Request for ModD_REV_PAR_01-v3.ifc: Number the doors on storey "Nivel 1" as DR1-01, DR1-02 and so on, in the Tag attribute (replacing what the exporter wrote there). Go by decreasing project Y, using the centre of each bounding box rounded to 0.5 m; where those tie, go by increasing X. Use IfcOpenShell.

First a look at what the model holds.

```python
import ifcopenshell
import ifcopenshell.util.element
import ifcopenshell.util.placement

model = ifcopenshell.open("ModD_REV_PAR_01-v3.ifc")
print(model.schema)
storey = next(s for s in model.by_type("IfcBuildingStorey") if s.Name == "Nivel 1")
doors = [e for e in ifcopenshell.util.element.get_decomposition(storey) if e.is_a("IfcDoor")]
for e in sorted(doors, key=lambda e: e.id()):
    origin = ifcopenshell.util.placement.get_local_placement(e.ObjectPlacement)[:3, 3]
    print(e.id(), e.Tag, e.Name, origin.round(2) + 0.0, sep=" | ")
```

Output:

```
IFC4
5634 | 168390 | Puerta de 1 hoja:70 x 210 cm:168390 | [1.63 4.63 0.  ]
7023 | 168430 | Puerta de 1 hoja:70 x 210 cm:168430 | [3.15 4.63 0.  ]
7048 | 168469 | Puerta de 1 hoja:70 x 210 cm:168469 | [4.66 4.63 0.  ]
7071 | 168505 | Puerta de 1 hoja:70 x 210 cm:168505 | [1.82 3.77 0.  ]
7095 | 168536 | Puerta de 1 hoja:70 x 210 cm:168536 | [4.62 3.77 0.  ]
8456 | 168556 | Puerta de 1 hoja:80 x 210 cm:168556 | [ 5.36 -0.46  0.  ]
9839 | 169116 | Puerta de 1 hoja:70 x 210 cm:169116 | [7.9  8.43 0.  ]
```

```python
import ifcopenshell
import ifcopenshell.geom
import ifcopenshell.util.element
import ifcopenshell.util.shape

model = ifcopenshell.open("ModD_REV_PAR_01-v3.ifc")
settings = ifcopenshell.geom.settings()
settings.set("use-world-coords", True)


def centre(element):
    shape = ifcopenshell.geom.create_shape(settings, element)
    return ifcopenshell.util.shape.get_bbox_centroid(shape.geometry)


storey = next(s for s in model.by_type("IfcBuildingStorey") if s.Name == "Nivel 1")
doors = [e for e in ifcopenshell.util.element.get_decomposition(storey) if e.is_a("IfcDoor")]

# Insertion points can sit at a corner or the storey origin, so sort by the geometry (in metres).
centres = {e: centre(e) for e in doors}
doors.sort(key=lambda e: (-round(centres[e][1] / 0.5), centres[e][0]))

for i, e in enumerate(doors, start=1):
    number = f"DR1-{i:02d}"
    e.Tag = number
    print(e.id(), number)

model.write("ModD_REV_PAR_01-v3_rev.ifc")
```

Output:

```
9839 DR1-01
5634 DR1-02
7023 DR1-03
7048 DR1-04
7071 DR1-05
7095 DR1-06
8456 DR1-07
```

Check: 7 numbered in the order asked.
